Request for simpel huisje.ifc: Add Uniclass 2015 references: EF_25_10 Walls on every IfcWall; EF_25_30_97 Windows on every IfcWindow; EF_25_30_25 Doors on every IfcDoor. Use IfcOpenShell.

First a look at what the model holds.

```python
import ifcopenshell

model = ifcopenshell.open("simpel huisje.ifc")
print(model.schema)
print("classifications:", [c.Name for c in model.by_type("IfcClassification")])
for ifc_class in ("IfcDoor", "IfcRoof", "IfcStair", "IfcWall", "IfcWindow"):
    print(ifc_class, len(model.by_type(ifc_class)))
```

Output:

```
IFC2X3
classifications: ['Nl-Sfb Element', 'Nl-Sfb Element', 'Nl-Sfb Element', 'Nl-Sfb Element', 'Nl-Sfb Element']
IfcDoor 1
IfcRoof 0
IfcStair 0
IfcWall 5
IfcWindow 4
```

```python
import ifcopenshell
import ifcopenshell.api.classification

model = ifcopenshell.open("simpel huisje.ifc")

# IFC2X3 requires Source and Edition and has no link from the project to the system.
system = model.create_entity("IfcClassification", Source="NBS", Edition="2015", Name="Uniclass 2015")

codes = {
    "IfcWall": ("EF_25_10", "Walls"),
    "IfcWindow": ("EF_25_30_97", "Windows"),
    "IfcDoor": ("EF_25_30_25", "Doors"),
}
for ifc_class, (code, name) in codes.items():
    products = model.by_type(ifc_class)
    ifcopenshell.api.classification.add_reference(
        model, products=products, classification=system, identification=code, name=name
    )
    print(code, len(products))

model.write("simpel huisje_rev.ifc")
```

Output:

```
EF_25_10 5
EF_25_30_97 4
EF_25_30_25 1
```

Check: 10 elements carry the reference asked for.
